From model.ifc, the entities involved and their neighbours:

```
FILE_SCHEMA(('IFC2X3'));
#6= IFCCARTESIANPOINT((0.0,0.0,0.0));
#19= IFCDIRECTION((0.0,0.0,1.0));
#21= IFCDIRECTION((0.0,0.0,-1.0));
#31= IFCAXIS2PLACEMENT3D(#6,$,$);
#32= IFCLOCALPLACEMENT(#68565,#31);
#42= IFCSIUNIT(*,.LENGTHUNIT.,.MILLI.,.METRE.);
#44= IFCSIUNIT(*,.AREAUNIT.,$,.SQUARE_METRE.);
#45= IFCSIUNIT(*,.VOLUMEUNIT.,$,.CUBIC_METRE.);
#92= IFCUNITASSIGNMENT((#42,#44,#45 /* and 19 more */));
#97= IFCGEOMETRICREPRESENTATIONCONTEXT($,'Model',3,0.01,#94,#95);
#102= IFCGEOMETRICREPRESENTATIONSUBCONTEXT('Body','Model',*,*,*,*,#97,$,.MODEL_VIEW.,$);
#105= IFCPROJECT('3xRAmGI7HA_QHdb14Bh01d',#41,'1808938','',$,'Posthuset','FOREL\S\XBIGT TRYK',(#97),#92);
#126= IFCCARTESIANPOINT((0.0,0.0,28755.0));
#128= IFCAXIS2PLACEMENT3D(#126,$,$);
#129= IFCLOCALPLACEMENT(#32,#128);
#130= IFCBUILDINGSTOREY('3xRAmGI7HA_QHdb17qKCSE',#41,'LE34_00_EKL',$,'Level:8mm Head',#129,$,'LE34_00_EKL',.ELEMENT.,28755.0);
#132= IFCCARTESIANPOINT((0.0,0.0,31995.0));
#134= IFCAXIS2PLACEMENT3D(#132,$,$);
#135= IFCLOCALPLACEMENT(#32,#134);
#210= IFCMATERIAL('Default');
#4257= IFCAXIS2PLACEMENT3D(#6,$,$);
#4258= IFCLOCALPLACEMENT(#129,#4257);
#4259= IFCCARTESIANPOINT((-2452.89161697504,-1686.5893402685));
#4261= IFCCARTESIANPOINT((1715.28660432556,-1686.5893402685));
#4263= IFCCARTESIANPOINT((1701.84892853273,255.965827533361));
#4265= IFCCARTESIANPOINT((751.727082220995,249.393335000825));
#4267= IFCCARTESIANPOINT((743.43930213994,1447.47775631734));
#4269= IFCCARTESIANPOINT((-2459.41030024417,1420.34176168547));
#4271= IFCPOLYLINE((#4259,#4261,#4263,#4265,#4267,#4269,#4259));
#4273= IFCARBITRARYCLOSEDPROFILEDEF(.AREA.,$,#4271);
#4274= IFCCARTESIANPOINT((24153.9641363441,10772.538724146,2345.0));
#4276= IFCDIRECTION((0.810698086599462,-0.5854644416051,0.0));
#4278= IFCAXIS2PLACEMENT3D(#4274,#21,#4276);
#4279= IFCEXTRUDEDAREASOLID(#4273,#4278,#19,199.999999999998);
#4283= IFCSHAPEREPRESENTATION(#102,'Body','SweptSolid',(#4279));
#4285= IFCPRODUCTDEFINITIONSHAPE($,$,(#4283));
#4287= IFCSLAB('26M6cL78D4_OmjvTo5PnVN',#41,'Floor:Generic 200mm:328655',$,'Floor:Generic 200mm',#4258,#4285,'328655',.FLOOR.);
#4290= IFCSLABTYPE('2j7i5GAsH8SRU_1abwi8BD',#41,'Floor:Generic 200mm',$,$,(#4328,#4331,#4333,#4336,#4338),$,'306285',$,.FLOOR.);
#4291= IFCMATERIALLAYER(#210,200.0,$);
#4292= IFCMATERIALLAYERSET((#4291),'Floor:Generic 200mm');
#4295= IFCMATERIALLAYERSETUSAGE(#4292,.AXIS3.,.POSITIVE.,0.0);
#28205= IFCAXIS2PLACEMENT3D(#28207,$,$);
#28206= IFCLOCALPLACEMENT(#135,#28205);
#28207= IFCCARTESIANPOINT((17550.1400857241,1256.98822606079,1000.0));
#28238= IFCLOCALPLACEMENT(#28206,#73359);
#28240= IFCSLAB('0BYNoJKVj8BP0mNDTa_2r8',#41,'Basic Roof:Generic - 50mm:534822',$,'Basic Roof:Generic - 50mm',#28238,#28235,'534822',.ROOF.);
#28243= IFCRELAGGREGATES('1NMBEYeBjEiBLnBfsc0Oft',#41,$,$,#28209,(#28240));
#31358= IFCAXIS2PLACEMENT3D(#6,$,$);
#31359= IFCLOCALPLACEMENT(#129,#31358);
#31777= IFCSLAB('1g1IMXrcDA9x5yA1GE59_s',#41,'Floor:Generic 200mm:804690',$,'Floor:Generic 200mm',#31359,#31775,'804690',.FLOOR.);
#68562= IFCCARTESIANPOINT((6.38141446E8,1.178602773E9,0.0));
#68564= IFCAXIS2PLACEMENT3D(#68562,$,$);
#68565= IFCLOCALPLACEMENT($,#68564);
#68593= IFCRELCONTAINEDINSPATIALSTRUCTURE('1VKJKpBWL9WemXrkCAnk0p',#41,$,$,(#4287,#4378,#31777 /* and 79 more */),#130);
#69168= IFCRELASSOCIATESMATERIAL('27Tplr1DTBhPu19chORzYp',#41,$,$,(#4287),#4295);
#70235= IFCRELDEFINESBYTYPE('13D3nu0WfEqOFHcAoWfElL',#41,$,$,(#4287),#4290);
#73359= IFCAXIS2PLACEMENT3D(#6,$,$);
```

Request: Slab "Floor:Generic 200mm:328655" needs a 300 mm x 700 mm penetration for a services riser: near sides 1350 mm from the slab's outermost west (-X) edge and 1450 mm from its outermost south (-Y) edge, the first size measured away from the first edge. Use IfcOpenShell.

```python
import numpy as np
import ifcopenshell
import ifcopenshell.api.feature
import ifcopenshell.api.geometry
import ifcopenshell.api.root
import ifcopenshell.geom
import ifcopenshell.util.placement
import ifcopenshell.util.representation
import ifcopenshell.util.shape
import ifcopenshell.util.unit

model = ifcopenshell.open("model.ifc")
unit_scale = ifcopenshell.util.unit.calculate_unit_scale(model)
settings = ifcopenshell.geom.settings()


def volume(element):
    """Net volume in cubic metres, openings subtracted."""
    shape = ifcopenshell.geom.create_shape(settings, element)
    return ifcopenshell.util.shape.get_volume(shape.geometry)


slab = model.by_guid("26M6cL78D4_OmjvTo5PnVN")
before = volume(slab)

# Extent in the slab's own axes, in metres. The edges named are its -X and -Y sides.
slab_shape = ifcopenshell.geom.create_shape(settings, slab)
vertices = ifcopenshell.util.shape.get_vertices(slab_shape.geometry)
x_min, y_min, bottom = vertices.min(axis=0)
top = vertices[:, 2].max()

opening = ifcopenshell.api.root.create_entity(model, ifc_class="IfcOpeningElement", name="Services riser opening")
context = ifcopenshell.util.representation.get_context(model, "Model", "Body", "MODEL_VIEW")
width, depth = 0.3, 0.7
outline = [(0.0, 0.0), (width, 0.0), (width, depth), (0.0, depth), (0.0, 0.0)]
# Overshoot both faces by 50 mm so the cut is clean.
shape = ifcopenshell.api.geometry.add_slab_representation(
    model, context=context, depth=top - bottom + 0.1, polyline=outline
)
ifcopenshell.api.geometry.assign_representation(model, product=opening, representation=shape)

matrix = ifcopenshell.util.placement.get_local_placement(slab.ObjectPlacement)
matrix[:, 3] = matrix @ np.append(np.array([x_min + 1.35, y_min + 1.45, bottom - 0.05]) / unit_scale, 1.0)
ifcopenshell.api.geometry.edit_object_placement(model, product=opening, matrix=matrix, is_si=False)
ifcopenshell.api.feature.add_feature(model, feature=opening, element=slab)

after = volume(slab)

print(f"slab volume {before:.3f} -> {after:.3f} m3")

model.write("model_edited.ifc")
```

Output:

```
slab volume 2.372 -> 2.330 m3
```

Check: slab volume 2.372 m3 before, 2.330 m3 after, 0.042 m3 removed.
